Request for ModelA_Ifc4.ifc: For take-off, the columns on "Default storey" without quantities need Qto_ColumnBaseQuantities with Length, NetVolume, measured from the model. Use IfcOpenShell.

First a look at what the model holds.

```python
import ifcopenshell
import ifcopenshell.util.element
import ifcopenshell.util.unit

model = ifcopenshell.open("ModelA_Ifc4.ifc")
print(model.schema)
for unit_type in ("LENGTHUNIT", "AREAUNIT", "VOLUMEUNIT"):
    print(unit_type, ifcopenshell.util.unit.calculate_unit_scale(model, unit_type))
storey = next(s for s in model.by_type("IfcBuildingStorey") if s.Name == "Default storey")
columns = [e for e in ifcopenshell.util.element.get_decomposition(storey) if e.is_a("IfcColumn")]
for e in sorted(columns, key=lambda e: e.id()):
    print(e.id(), e.is_a(), e.Name, list(ifcopenshell.util.element.get_psets(e, qtos_only=True)), sep=" | ")
```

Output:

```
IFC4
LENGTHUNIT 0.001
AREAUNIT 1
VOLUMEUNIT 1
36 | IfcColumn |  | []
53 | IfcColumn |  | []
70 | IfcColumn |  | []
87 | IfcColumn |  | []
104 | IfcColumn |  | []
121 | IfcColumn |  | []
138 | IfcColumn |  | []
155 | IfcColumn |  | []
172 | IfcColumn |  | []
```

```python
import ifcopenshell
import ifcopenshell.api.pset
import ifcopenshell.geom
import ifcopenshell.util.element
import ifcopenshell.util.shape
import ifcopenshell.util.unit

model = ifcopenshell.open("ModelA_Ifc4.ifc")
unit_scale = ifcopenshell.util.unit.calculate_unit_scale(model)
volume_scale = ifcopenshell.util.unit.calculate_unit_scale(model, "VOLUMEUNIT")
settings = ifcopenshell.geom.settings()

storey = next(s for s in model.by_type("IfcBuildingStorey") if s.Name == "Default storey")
columns = [e for e in ifcopenshell.util.element.get_decomposition(storey) if e.is_a("IfcColumn")]

for e in sorted(columns, key=lambda e: e.id()):
    if ifcopenshell.util.element.get_psets(e, qtos_only=True, should_inherit=False):
        continue
    # Geometry comes back in metres, in the element's own axes.
    shape = ifcopenshell.geom.create_shape(settings, e)
    values = {
        "Length": ifcopenshell.util.shape.get_z(shape.geometry) / unit_scale,
        "NetVolume": ifcopenshell.util.shape.get_volume(shape.geometry) / volume_scale,
    }
    qto = ifcopenshell.api.pset.add_qto(model, product=e, name="Qto_ColumnBaseQuantities")
    ifcopenshell.api.pset.edit_qto(model, qto=qto, properties=values)
    print(e.id(), {k: round(v, 3) for k, v in values.items()})

model.write("ModelA_Ifc4-out.ifc")
```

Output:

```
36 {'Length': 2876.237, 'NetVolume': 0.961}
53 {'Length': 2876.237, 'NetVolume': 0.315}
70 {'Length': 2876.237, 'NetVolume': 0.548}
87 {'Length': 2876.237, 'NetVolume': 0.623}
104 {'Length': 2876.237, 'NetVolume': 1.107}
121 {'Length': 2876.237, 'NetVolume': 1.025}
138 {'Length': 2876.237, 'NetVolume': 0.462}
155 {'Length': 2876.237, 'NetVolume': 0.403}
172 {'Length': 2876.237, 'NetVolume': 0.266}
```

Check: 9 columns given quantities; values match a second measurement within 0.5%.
